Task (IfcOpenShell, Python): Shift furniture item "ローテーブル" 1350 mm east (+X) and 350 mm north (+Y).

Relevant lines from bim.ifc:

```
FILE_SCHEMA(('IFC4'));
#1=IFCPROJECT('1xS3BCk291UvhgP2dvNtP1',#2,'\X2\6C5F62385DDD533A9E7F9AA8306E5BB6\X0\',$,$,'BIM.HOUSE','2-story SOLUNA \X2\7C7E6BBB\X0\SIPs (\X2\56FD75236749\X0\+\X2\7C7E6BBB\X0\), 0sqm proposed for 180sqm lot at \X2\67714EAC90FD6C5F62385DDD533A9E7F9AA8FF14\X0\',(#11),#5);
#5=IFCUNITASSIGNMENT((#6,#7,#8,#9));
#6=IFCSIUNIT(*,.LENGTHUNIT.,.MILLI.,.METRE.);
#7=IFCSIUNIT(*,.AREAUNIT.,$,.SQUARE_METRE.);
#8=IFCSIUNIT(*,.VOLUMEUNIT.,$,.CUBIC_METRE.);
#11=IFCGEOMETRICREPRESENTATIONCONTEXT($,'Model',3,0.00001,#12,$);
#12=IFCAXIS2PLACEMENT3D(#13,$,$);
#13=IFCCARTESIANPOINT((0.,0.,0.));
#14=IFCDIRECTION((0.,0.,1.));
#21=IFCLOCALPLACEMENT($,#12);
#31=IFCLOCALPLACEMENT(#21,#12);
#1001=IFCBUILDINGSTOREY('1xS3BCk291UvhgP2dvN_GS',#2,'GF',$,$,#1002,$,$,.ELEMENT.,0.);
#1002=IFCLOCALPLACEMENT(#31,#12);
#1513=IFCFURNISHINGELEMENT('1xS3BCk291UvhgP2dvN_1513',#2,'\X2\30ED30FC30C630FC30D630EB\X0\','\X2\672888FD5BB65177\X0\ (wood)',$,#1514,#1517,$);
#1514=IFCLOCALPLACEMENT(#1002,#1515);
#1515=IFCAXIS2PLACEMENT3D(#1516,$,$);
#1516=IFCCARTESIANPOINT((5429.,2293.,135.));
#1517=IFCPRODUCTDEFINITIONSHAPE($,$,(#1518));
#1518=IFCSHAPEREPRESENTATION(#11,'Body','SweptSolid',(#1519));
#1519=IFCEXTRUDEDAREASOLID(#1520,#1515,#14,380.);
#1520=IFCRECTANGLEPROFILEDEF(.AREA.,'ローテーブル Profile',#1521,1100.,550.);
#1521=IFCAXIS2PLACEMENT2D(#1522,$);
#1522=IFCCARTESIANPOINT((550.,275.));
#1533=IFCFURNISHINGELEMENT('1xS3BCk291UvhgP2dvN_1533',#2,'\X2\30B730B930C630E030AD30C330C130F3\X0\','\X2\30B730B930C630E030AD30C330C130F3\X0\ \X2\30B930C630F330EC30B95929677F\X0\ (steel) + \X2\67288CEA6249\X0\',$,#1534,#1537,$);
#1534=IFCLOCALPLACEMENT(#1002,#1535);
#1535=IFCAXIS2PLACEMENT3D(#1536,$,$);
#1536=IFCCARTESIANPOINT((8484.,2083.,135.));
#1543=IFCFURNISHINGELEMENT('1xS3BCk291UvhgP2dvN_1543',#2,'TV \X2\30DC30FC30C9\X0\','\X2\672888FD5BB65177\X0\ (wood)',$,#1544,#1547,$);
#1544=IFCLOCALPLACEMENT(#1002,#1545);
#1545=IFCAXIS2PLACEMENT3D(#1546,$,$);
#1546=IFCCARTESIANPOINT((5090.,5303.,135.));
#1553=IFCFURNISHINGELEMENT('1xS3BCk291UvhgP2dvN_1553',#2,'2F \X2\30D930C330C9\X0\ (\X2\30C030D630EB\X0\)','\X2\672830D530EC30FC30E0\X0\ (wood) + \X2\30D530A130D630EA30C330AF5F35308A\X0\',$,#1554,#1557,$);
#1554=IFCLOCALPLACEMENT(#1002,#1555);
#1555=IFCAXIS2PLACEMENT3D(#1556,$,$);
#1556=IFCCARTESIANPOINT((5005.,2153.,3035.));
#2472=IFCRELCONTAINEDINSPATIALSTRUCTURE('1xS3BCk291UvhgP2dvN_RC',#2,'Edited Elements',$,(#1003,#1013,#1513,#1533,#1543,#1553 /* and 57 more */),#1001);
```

```python
import ifcopenshell
import ifcopenshell.api.geometry
import ifcopenshell.util.placement
import ifcopenshell.util.unit

model = ifcopenshell.open("bim.ifc")
unit_scale = ifcopenshell.util.unit.calculate_unit_scale(model)

item = model.by_id(1513)
matrix = ifcopenshell.util.placement.get_local_placement(item.ObjectPlacement)
matrix[0, 3] += 1.35 / unit_scale
matrix[1, 3] += 0.35 / unit_scale
ifcopenshell.api.geometry.edit_object_placement(model, product=item, matrix=matrix, is_si=False)

print(ifcopenshell.util.placement.get_local_placement(item.ObjectPlacement).round(3) + 0.0)

model.write("bim_v2.ifc")
```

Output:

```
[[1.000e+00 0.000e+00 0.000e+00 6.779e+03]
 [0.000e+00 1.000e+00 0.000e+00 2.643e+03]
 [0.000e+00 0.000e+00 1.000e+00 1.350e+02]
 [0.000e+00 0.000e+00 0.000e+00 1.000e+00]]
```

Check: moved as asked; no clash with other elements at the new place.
